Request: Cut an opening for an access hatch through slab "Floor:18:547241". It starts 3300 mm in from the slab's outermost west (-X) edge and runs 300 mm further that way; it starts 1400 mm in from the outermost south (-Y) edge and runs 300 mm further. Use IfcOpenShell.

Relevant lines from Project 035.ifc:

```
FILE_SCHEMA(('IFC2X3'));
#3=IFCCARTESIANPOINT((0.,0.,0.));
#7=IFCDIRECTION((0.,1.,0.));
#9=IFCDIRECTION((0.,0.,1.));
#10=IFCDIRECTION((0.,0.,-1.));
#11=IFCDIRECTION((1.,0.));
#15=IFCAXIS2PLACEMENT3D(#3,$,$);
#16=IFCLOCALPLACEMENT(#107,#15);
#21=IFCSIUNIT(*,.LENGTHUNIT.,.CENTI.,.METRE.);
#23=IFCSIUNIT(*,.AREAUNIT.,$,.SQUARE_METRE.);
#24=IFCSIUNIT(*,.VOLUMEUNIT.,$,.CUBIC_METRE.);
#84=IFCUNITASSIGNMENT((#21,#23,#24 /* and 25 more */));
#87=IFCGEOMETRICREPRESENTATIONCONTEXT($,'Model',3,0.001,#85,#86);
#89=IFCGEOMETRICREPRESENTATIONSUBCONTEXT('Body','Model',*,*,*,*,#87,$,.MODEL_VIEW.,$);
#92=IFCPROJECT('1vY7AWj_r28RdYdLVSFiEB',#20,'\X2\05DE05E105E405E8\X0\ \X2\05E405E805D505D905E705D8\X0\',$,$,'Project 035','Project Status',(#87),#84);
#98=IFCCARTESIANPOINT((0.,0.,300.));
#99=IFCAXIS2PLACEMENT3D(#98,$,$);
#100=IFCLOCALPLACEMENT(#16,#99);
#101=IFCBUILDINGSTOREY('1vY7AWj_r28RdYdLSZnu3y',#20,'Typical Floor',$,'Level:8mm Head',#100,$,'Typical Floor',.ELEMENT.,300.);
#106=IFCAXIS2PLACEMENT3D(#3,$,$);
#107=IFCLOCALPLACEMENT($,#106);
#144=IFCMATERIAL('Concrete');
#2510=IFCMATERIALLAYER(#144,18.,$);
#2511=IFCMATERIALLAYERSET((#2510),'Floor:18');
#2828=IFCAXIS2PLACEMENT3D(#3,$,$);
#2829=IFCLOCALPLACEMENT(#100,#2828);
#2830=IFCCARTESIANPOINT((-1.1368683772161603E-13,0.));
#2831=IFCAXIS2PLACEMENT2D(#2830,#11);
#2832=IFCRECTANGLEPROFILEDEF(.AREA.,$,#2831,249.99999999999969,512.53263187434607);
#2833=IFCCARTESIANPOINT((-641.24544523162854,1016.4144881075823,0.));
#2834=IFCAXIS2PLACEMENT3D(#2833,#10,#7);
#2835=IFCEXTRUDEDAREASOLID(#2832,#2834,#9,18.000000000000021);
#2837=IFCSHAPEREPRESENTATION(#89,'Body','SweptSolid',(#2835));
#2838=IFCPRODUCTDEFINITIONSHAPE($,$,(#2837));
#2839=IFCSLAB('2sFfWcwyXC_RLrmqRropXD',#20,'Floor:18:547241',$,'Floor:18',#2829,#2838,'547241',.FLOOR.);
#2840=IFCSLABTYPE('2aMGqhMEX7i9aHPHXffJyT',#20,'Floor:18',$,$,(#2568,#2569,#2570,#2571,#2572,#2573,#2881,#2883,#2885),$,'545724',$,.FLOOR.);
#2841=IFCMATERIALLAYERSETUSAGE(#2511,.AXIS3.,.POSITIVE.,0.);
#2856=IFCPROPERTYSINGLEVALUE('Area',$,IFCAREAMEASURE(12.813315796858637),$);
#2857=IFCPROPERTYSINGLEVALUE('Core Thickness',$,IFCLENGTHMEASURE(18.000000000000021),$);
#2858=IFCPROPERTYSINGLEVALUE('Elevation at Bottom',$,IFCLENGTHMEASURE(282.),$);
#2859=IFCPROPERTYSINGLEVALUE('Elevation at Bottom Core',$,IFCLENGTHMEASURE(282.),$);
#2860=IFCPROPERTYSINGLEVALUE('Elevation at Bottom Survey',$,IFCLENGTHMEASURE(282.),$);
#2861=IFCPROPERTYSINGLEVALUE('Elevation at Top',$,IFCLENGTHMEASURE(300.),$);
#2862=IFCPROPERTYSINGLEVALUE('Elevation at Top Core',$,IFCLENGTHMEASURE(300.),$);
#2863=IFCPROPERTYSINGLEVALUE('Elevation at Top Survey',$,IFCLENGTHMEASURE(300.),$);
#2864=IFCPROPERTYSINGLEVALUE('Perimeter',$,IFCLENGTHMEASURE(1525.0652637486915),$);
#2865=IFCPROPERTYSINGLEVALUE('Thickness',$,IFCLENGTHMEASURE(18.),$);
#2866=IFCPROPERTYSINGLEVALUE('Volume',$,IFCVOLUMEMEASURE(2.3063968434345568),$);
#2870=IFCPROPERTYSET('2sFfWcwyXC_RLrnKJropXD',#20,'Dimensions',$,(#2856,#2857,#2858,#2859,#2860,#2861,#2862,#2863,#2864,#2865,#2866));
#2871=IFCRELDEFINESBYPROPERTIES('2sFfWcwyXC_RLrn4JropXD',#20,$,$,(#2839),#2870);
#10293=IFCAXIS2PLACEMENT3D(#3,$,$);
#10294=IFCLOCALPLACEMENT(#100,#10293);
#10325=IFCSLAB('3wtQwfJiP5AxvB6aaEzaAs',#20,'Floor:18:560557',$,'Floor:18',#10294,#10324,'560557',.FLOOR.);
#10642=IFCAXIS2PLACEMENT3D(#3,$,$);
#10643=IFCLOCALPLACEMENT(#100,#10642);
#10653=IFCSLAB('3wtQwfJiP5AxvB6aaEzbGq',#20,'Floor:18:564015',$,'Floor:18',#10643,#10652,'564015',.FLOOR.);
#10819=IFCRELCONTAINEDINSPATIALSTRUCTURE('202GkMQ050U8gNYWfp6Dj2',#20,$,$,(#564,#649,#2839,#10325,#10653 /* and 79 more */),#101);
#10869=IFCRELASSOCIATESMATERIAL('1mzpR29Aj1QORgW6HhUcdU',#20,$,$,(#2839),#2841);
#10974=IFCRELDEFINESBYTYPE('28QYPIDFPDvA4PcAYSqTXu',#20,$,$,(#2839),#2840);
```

```python
import numpy as np
import ifcopenshell
import ifcopenshell.api.feature
import ifcopenshell.api.geometry
import ifcopenshell.api.pset
import ifcopenshell.api.root
import ifcopenshell.geom
import ifcopenshell.util.element
import ifcopenshell.util.placement
import ifcopenshell.util.representation
import ifcopenshell.util.shape
import ifcopenshell.util.unit

model = ifcopenshell.open("Project 035.ifc")
unit_scale = ifcopenshell.util.unit.calculate_unit_scale(model)
area_scale = ifcopenshell.util.unit.calculate_unit_scale(model, "AREAUNIT")
volume_scale = ifcopenshell.util.unit.calculate_unit_scale(model, "VOLUMEUNIT")
settings = ifcopenshell.geom.settings()


def volume(element):
    """Net volume in cubic metres, openings subtracted."""
    shape = ifcopenshell.geom.create_shape(settings, element)
    return ifcopenshell.util.shape.get_volume(shape.geometry)


slab = model.by_guid("2sFfWcwyXC_RLrmqRropXD")
before = volume(slab)

# Extent in the slab's own axes, in metres. The edges named are its -X and -Y sides.
slab_shape = ifcopenshell.geom.create_shape(settings, slab)
vertices = ifcopenshell.util.shape.get_vertices(slab_shape.geometry)
x_min, y_min, bottom = vertices.min(axis=0)
top = vertices[:, 2].max()

opening = ifcopenshell.api.root.create_entity(model, ifc_class="IfcOpeningElement", name="Access hatch opening")
context = ifcopenshell.util.representation.get_context(model, "Model", "Body", "MODEL_VIEW")
width, depth = 0.3, 0.3
outline = [(0.0, 0.0), (width, 0.0), (width, depth), (0.0, depth), (0.0, 0.0)]
# Overshoot both faces by 50 mm so the cut is clean.
shape = ifcopenshell.api.geometry.add_slab_representation(
    model, context=context, depth=top - bottom + 0.1, polyline=outline
)
ifcopenshell.api.geometry.assign_representation(model, product=opening, representation=shape)

matrix = ifcopenshell.util.placement.get_local_placement(slab.ObjectPlacement)
matrix[:, 3] = matrix @ np.append(np.array([x_min + 3.3, y_min + 1.4, bottom - 0.05]) / unit_scale, 1.0)
ifcopenshell.api.geometry.edit_object_placement(model, product=opening, matrix=matrix, is_si=False)
ifcopenshell.api.feature.add_feature(model, feature=opening, element=slab)

after = volume(slab)

# Update the slab's stored quantities.
pset = model.by_id(ifcopenshell.util.element.get_pset(slab, "Dimensions", should_inherit=False)["id"])
ifcopenshell.api.pset.edit_pset(model, pset=pset, properties={
    "Area": model.create_entity("IfcAreaMeasure", after / (top - bottom) / area_scale),
    "Volume": model.create_entity("IfcVolumeMeasure", after / volume_scale),
})

print(f"slab volume {before:.3f} -> {after:.3f} m3")

model.write("Project 035_v2.ifc")
```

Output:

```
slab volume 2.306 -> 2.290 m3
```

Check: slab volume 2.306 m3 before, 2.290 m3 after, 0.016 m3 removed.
